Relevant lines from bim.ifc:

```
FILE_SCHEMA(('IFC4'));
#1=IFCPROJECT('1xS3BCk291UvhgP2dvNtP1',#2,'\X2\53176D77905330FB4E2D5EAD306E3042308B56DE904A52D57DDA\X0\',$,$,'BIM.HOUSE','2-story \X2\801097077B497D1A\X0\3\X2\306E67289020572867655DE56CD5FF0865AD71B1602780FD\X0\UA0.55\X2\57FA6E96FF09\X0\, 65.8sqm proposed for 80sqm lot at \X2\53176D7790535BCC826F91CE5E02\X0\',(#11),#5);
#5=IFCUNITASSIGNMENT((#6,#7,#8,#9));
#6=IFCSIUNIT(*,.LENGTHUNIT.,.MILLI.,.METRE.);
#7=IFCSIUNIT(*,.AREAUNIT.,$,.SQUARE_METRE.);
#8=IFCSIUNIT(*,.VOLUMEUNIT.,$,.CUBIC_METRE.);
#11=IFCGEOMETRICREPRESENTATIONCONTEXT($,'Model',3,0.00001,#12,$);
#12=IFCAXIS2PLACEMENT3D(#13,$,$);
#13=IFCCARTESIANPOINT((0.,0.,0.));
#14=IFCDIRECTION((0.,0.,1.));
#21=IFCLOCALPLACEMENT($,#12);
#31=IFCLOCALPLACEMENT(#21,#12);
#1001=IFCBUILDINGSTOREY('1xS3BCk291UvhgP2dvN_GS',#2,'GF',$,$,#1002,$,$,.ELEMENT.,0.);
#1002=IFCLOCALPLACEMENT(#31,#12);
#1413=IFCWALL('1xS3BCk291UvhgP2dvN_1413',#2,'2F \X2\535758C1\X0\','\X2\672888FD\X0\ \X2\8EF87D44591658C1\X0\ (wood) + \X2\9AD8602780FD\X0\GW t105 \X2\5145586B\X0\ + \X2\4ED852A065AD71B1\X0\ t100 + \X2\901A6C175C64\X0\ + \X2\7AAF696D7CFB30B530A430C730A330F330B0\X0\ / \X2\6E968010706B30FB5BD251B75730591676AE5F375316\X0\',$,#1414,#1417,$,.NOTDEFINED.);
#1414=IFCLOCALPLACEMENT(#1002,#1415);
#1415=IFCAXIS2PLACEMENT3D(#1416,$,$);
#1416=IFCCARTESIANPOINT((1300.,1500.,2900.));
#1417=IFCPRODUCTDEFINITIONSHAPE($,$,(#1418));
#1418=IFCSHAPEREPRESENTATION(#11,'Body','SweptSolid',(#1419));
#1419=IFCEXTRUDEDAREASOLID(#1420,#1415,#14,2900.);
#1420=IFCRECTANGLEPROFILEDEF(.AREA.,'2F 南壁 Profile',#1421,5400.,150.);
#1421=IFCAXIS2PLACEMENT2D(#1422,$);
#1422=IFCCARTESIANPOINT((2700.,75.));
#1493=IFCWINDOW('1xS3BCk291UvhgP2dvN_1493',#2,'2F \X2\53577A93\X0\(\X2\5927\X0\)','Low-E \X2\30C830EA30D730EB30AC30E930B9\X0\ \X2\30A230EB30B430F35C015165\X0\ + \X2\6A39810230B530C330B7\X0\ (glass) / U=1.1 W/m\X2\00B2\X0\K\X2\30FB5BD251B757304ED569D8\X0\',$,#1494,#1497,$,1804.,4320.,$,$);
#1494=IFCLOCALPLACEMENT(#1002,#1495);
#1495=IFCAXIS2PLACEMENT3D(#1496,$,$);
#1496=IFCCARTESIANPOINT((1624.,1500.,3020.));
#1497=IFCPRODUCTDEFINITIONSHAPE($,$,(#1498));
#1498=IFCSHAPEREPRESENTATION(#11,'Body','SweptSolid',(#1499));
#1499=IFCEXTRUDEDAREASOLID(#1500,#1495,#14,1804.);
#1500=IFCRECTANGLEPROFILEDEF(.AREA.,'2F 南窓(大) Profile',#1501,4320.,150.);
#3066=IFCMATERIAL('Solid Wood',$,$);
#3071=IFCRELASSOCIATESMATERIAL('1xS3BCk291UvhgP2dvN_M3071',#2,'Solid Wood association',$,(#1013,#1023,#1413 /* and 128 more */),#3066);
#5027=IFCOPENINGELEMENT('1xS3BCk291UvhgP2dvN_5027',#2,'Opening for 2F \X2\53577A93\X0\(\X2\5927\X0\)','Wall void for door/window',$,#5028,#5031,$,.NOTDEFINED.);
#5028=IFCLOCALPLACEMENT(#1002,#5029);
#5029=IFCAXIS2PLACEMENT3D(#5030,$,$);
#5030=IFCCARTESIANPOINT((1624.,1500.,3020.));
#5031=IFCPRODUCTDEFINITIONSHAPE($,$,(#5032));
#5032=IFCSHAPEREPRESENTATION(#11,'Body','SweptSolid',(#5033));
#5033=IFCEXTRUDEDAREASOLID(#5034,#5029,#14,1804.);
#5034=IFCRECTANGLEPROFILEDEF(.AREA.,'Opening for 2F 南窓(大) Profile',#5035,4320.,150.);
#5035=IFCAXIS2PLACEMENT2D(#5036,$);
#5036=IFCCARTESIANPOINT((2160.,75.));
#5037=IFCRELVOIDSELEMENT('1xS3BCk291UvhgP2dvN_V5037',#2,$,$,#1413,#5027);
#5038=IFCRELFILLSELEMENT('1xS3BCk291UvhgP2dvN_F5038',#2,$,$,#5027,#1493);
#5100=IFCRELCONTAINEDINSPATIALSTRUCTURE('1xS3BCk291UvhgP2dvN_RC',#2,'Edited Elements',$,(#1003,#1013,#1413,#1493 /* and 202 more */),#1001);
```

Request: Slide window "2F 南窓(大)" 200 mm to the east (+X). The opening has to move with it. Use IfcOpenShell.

```python
import ifcopenshell
import ifcopenshell.api.geometry
import ifcopenshell.util.placement

model = ifcopenshell.open("bim.ifc")

window = model.by_guid("1xS3BCk291UvhgP2dvN_1493")
opening = window.FillsVoids[0].RelatingOpeningElement
wall = opening.VoidsElements[0].RelatingBuildingElement

wall_matrix = ifcopenshell.util.placement.get_local_placement(wall.ObjectPlacement)
shift = wall_matrix[:3, 0] * 200.0
before = ifcopenshell.util.placement.get_local_placement(window.ObjectPlacement)[:3, 3].copy()

# The window is not placed relative to its opening, so move both.
for product in (opening, window):
    matrix = ifcopenshell.util.placement.get_local_placement(product.ObjectPlacement)
    matrix[:3, 3] += shift
    ifcopenshell.api.geometry.edit_object_placement(model, product=product, matrix=matrix, is_si=False)

after = ifcopenshell.util.placement.get_local_placement(window.ObjectPlacement)[:3, 3]
print("window moved by", (after - before).round(3) + 0.0)

model.write("bim_rev.ifc")
```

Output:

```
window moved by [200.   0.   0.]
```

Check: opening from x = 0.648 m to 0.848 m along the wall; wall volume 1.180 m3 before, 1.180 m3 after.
